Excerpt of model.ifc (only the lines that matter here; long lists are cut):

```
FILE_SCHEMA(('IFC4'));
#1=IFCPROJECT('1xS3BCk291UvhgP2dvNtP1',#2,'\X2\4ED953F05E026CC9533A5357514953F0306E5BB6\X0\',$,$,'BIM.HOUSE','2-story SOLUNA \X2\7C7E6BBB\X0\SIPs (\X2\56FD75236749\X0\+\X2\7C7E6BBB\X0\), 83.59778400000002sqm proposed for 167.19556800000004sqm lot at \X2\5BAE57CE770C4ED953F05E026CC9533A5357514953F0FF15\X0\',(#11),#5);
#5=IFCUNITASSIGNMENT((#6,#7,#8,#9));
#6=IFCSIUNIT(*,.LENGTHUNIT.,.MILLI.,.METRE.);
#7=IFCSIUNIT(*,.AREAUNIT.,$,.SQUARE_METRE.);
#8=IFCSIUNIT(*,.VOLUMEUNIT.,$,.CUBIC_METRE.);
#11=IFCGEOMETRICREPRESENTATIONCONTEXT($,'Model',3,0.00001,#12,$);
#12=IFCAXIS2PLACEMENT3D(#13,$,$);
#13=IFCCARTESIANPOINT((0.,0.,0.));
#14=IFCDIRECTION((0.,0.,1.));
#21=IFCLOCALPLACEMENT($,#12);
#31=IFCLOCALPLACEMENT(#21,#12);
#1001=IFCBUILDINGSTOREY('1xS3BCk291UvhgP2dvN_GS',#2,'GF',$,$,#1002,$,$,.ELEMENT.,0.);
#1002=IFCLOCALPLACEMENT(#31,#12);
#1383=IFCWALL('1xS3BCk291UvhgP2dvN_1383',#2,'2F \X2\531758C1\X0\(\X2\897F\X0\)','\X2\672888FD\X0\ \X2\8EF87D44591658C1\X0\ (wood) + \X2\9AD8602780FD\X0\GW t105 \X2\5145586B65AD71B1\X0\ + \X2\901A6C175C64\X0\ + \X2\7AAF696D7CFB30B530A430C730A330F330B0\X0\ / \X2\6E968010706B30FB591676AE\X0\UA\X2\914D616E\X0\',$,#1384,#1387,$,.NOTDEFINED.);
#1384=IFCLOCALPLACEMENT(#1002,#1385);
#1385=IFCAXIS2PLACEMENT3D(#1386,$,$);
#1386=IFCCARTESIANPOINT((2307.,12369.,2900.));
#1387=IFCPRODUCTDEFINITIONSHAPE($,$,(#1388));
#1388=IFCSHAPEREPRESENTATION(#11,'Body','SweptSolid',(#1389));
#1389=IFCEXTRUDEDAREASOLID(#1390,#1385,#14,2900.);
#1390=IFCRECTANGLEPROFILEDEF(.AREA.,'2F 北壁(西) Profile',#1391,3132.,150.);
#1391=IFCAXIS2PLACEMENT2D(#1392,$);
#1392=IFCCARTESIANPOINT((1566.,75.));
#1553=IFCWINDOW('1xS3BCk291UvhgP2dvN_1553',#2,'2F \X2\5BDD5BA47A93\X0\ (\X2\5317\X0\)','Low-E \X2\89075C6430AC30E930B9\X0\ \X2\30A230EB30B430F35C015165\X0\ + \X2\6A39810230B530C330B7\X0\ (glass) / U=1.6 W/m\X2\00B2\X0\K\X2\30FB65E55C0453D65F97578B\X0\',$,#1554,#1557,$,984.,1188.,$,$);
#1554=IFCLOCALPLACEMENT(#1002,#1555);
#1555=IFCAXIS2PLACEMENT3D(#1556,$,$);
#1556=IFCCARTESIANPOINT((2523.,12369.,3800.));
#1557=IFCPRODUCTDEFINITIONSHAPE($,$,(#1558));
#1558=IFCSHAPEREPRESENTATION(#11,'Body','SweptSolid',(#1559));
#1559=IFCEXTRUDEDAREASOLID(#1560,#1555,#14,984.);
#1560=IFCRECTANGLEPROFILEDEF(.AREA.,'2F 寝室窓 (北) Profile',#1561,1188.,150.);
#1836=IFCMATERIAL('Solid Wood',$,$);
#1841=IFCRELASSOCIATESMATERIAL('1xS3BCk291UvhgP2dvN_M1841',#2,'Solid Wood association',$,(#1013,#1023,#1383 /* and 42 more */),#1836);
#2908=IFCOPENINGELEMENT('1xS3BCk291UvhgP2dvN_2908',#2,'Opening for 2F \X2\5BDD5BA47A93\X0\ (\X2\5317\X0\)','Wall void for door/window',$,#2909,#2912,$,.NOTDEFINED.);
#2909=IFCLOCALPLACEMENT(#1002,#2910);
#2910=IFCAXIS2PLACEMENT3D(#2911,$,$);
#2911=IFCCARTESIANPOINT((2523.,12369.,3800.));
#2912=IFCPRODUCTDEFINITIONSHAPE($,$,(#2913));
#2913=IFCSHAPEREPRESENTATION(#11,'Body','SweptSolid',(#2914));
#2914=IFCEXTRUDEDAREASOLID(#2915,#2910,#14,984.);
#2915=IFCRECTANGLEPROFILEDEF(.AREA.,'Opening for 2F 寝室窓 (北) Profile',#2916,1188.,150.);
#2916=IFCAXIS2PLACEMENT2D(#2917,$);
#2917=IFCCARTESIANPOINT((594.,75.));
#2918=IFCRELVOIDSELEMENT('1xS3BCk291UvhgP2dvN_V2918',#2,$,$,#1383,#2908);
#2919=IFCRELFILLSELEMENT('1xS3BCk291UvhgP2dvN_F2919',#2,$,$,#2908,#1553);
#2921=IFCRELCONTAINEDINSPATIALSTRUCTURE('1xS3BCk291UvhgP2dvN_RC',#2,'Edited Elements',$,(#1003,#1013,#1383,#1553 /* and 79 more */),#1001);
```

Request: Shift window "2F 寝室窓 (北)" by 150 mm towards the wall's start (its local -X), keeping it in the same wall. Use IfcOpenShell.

```python
import ifcopenshell
import ifcopenshell.api.geometry
import ifcopenshell.util.placement

model = ifcopenshell.open("model.ifc")

window = model.by_guid("1xS3BCk291UvhgP2dvN_1553")
opening = window.FillsVoids[0].RelatingOpeningElement
wall = opening.VoidsElements[0].RelatingBuildingElement

wall_matrix = ifcopenshell.util.placement.get_local_placement(wall.ObjectPlacement)
shift = wall_matrix[:3, 0] * -150.0
before = ifcopenshell.util.placement.get_local_placement(window.ObjectPlacement)[:3, 3].copy()

# The window is not placed relative to its opening, so move both.
for product in (opening, window):
    matrix = ifcopenshell.util.placement.get_local_placement(product.ObjectPlacement)
    matrix[:3, 3] += shift
    ifcopenshell.api.geometry.edit_object_placement(model, product=product, matrix=matrix, is_si=False)

after = ifcopenshell.util.placement.get_local_placement(window.ObjectPlacement)[:3, 3]
print("window moved by", (after - before).round(3) + 0.0)

model.write("model_rev.ifc")
```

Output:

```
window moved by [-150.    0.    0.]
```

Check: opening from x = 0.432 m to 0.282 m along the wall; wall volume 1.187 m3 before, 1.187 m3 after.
